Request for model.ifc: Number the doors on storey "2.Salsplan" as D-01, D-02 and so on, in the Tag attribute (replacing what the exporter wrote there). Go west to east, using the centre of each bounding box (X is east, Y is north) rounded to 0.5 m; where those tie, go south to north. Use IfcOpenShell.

First a look at what the model holds.

```python
import ifcopenshell
import ifcopenshell.util.element
import ifcopenshell.util.placement

model = ifcopenshell.open("model.ifc")
print(model.schema)
storey = next(s for s in model.by_type("IfcBuildingStorey") if s.Name == "2.Salsplan")
doors = [e for e in ifcopenshell.util.element.get_decomposition(storey) if e.is_a("IfcDoor")]
for e in sorted(doors, key=lambda e: e.id()):
    origin = ifcopenshell.util.placement.get_local_placement(e.ObjectPlacement)[:3, 3]
    print(e.id(), e.Tag, e.Name, origin.round(2) + 0.0, sep=" | ")
```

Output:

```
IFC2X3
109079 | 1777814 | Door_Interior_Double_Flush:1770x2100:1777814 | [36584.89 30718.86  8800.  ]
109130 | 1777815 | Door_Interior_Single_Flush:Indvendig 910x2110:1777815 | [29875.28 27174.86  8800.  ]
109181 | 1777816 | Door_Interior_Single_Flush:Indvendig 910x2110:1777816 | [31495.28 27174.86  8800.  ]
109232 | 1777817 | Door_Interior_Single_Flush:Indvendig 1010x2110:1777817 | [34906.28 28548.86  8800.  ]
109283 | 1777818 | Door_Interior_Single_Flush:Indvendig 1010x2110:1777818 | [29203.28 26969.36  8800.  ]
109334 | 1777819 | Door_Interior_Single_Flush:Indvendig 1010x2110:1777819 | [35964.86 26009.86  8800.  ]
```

```python
import ifcopenshell
import ifcopenshell.geom
import ifcopenshell.util.element
import ifcopenshell.util.shape

model = ifcopenshell.open("model.ifc")
settings = ifcopenshell.geom.settings()
settings.set("use-world-coords", True)


def centre(element):
    shape = ifcopenshell.geom.create_shape(settings, element)
    return ifcopenshell.util.shape.get_bbox_centroid(shape.geometry)


storey = next(s for s in model.by_type("IfcBuildingStorey") if s.Name == "2.Salsplan")
doors = [e for e in ifcopenshell.util.element.get_decomposition(storey) if e.is_a("IfcDoor")]

# Insertion points can sit at a corner or the storey origin, so sort by the geometry (in metres).
centres = {e: centre(e) for e in doors}
doors.sort(key=lambda e: (round(centres[e][0] / 0.5), centres[e][1]))

for i, e in enumerate(doors, start=1):
    number = f"D-{i:02d}"
    e.Tag = number
    print(e.id(), number)

model.write("model_updated.ifc")
```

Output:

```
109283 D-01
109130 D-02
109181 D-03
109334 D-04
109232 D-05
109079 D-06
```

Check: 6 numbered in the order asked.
